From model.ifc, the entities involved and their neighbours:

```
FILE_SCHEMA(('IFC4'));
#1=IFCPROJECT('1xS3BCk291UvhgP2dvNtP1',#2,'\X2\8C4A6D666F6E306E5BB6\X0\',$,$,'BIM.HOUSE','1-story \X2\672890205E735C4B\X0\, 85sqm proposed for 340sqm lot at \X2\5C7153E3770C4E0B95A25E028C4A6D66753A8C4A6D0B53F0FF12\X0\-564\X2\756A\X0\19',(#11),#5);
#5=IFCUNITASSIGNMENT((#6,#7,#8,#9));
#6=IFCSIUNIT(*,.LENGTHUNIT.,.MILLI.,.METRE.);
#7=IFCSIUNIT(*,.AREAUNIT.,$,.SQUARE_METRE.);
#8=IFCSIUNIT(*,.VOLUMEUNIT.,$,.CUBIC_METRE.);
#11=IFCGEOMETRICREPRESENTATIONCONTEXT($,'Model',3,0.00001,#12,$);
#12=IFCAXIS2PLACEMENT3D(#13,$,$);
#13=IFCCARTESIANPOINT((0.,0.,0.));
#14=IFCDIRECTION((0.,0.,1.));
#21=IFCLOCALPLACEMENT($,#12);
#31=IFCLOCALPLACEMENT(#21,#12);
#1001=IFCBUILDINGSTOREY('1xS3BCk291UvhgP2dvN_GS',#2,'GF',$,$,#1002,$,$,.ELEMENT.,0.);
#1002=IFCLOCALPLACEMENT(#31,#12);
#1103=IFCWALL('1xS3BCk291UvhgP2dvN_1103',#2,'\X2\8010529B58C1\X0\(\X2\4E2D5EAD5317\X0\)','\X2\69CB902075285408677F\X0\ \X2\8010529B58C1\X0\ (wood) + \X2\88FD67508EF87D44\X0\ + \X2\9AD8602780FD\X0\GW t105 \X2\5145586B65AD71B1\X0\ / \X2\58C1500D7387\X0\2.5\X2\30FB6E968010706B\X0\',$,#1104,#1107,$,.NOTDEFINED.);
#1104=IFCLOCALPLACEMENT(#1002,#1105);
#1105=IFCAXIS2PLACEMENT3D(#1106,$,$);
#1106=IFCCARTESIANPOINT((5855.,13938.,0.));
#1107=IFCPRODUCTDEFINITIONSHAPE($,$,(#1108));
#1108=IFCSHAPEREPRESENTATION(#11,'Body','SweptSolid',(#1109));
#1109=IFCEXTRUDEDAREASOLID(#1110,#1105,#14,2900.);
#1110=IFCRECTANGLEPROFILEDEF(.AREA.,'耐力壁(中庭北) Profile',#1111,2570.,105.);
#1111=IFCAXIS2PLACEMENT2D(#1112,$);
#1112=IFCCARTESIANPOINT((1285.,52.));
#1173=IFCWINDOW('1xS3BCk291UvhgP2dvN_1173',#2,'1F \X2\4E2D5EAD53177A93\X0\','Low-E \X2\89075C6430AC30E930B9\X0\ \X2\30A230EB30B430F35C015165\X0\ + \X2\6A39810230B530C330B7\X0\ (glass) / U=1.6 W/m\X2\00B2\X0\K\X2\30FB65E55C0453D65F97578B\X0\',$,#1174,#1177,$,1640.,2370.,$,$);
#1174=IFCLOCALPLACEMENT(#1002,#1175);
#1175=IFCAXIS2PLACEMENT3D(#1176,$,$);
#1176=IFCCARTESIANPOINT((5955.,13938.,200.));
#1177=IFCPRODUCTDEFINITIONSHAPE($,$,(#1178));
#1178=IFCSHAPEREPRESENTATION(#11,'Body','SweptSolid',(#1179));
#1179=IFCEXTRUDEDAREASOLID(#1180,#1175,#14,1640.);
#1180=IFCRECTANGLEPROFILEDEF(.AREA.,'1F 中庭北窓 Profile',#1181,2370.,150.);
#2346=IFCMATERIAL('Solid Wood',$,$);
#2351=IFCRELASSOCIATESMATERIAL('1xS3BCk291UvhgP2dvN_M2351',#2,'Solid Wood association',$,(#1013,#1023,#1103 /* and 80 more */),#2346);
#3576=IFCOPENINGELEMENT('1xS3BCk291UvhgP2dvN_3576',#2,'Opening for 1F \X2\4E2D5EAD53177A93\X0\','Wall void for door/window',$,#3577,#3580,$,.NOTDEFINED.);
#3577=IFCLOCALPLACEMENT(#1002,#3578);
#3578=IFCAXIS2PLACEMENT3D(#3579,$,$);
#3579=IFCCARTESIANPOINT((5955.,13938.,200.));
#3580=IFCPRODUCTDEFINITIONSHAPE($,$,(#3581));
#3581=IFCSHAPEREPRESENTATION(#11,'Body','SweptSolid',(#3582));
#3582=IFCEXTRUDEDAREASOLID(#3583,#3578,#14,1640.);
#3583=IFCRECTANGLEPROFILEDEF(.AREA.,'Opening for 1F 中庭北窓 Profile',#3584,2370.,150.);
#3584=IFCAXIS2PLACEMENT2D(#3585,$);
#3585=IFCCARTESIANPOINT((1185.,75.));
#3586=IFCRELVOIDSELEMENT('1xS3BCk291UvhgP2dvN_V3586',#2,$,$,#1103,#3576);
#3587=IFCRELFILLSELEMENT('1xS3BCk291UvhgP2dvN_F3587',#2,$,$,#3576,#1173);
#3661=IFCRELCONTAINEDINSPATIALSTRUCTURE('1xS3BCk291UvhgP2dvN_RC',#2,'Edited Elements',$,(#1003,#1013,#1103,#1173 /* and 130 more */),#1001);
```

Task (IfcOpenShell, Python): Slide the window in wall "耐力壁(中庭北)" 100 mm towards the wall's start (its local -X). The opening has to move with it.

```python
import ifcopenshell
import ifcopenshell.api.geometry
import ifcopenshell.util.placement
import ifcopenshell.util.unit

model = ifcopenshell.open("model.ifc")
unit_scale = ifcopenshell.util.unit.calculate_unit_scale(model)

window = model.by_guid("1xS3BCk291UvhgP2dvN_1173")
opening = window.FillsVoids[0].RelatingOpeningElement
wall = opening.VoidsElements[0].RelatingBuildingElement

wall_matrix = ifcopenshell.util.placement.get_local_placement(wall.ObjectPlacement)
shift = wall_matrix[:3, 0] * -0.1 / unit_scale
before = ifcopenshell.util.placement.get_local_placement(window.ObjectPlacement)[:3, 3].copy()

# The window is not placed relative to its opening, so move both.
for product in (opening, window):
    matrix = ifcopenshell.util.placement.get_local_placement(product.ObjectPlacement)
    matrix[:3, 3] += shift
    ifcopenshell.api.geometry.edit_object_placement(model, product=product, matrix=matrix, is_si=False)

after = ifcopenshell.util.placement.get_local_placement(window.ObjectPlacement)[:3, 3]
print("window moved by", (after - before).round(3) + 0.0)

model.write("model_updated.ifc")
```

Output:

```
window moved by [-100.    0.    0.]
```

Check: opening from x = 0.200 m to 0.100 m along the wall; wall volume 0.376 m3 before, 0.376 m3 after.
